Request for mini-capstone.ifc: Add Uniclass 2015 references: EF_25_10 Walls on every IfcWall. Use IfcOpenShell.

First a look at what the model holds.

```python
import ifcopenshell

model = ifcopenshell.open("mini-capstone.ifc")
print(model.schema)
print("classifications:", [c.Name for c in model.by_type("IfcClassification")])
for ifc_class in ("IfcDoor", "IfcRoof", "IfcStair", "IfcWall", "IfcWindow"):
    print(ifc_class, len(model.by_type(ifc_class)))
```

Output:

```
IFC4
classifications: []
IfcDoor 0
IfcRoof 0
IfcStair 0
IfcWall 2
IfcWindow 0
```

```python
import ifcopenshell
import ifcopenshell.api.classification

model = ifcopenshell.open("mini-capstone.ifc")

system = ifcopenshell.api.classification.add_classification(model, classification="Uniclass 2015")

codes = {
    "IfcWall": ("EF_25_10", "Walls"),
}
for ifc_class, (code, name) in codes.items():
    products = model.by_type(ifc_class)
    ifcopenshell.api.classification.add_reference(
        model, products=products, classification=system, identification=code, name=name
    )
    print(code, len(products))

model.write("mini-capstone_edited.ifc")
```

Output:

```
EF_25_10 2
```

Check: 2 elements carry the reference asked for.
